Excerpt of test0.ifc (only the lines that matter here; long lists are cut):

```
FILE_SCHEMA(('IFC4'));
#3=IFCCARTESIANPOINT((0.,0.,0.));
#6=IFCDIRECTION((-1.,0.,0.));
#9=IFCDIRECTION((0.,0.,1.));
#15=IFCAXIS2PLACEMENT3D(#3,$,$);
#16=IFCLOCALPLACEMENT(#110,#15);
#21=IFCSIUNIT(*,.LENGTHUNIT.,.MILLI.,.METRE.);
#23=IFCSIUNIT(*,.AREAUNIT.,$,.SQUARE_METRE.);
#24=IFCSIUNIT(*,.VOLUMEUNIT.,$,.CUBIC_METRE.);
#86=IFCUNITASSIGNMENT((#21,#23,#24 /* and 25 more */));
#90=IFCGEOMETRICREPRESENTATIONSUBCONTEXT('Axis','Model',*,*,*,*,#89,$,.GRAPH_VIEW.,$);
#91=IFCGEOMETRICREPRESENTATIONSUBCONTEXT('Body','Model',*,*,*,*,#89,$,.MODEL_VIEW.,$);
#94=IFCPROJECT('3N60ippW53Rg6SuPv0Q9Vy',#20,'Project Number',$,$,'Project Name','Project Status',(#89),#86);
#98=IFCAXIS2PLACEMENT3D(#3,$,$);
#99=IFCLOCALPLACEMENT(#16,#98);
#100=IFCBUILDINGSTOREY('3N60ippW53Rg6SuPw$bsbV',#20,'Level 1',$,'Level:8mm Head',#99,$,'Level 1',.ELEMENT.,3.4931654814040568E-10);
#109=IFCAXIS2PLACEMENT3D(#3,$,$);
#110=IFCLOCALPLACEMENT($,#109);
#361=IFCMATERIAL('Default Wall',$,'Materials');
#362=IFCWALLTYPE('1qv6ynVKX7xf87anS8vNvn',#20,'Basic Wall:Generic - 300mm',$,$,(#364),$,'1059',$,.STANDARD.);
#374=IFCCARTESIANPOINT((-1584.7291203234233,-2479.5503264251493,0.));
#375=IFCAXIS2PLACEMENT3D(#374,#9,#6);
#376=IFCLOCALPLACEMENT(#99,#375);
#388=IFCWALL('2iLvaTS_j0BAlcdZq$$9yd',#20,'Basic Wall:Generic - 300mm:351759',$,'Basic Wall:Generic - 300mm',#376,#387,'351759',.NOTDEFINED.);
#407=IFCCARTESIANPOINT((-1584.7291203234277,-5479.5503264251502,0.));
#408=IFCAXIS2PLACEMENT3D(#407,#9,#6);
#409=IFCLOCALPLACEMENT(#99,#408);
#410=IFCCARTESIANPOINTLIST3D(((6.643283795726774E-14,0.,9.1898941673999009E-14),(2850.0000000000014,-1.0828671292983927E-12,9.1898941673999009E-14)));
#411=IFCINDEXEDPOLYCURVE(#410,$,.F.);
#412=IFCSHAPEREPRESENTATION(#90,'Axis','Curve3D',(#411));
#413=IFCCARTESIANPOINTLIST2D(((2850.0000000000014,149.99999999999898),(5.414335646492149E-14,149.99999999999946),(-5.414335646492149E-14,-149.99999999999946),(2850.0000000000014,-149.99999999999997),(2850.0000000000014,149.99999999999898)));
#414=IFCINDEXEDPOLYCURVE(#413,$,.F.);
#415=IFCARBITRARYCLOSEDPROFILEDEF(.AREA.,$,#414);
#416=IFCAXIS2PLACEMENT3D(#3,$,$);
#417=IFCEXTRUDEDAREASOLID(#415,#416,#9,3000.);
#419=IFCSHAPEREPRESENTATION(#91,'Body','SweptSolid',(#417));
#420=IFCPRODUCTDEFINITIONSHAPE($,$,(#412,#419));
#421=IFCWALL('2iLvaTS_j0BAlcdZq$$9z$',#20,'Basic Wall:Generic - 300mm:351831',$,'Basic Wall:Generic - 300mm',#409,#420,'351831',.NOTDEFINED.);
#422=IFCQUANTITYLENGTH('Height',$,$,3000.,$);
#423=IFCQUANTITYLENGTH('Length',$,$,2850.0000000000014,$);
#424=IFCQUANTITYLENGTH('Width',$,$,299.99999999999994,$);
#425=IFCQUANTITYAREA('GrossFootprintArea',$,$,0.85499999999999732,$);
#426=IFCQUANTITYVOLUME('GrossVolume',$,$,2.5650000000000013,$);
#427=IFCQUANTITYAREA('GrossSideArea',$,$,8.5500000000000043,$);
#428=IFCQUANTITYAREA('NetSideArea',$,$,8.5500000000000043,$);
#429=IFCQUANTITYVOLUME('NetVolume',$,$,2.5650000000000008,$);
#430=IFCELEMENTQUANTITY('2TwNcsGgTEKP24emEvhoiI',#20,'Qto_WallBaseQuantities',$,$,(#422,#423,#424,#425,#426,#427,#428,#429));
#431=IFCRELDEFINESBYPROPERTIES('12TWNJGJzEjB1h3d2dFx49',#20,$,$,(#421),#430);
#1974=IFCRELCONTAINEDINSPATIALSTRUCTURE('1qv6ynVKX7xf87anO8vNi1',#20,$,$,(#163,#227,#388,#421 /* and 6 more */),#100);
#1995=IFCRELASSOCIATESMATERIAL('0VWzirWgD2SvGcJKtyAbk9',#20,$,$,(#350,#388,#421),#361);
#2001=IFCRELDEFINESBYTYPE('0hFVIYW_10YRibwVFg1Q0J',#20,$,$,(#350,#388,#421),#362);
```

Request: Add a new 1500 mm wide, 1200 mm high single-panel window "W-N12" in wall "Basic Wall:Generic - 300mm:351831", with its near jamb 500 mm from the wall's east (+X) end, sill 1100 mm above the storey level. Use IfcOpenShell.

```python
import numpy as np
import ifcopenshell
import ifcopenshell.api.feature
import ifcopenshell.api.geometry
import ifcopenshell.api.pset
import ifcopenshell.api.root
import ifcopenshell.api.spatial
import ifcopenshell.geom
import ifcopenshell.util.element
import ifcopenshell.util.placement
import ifcopenshell.util.representation
import ifcopenshell.util.shape
import ifcopenshell.util.unit

model = ifcopenshell.open("test0.ifc")
unit_scale = ifcopenshell.util.unit.calculate_unit_scale(model)
area_scale = ifcopenshell.util.unit.calculate_unit_scale(model, "AREAUNIT")
volume_scale = ifcopenshell.util.unit.calculate_unit_scale(model, "VOLUMEUNIT")
settings = ifcopenshell.geom.settings()


def volume(element):
    """Net volume in cubic metres, openings subtracted."""
    shape = ifcopenshell.geom.create_shape(settings, element)
    return ifcopenshell.util.shape.get_volume(shape.geometry)


wall = model.by_guid("2iLvaTS_j0BAlcdZq$$9z$")
storey = ifcopenshell.util.element.get_container(wall, ifc_class="IfcBuildingStorey")
context = ifcopenshell.util.representation.get_context(model, "Model", "Body", "MODEL_VIEW")
before = volume(wall)

width, height, from_end, sill = 1.5, 1.2, 0.5, 1.1  # metres

# The wall runs along its own X axis, and the end named is its -X end.
wall_shape = ifcopenshell.geom.create_shape(settings, wall)
x, y, z = ifcopenshell.util.shape.get_vertices(wall_shape.geometry).T
start = x.min() + from_end
face, thickness = float(y.min()), float(y.max() - y.min())
wall_matrix = ifcopenshell.util.placement.get_local_placement(wall.ObjectPlacement)
level = ifcopenshell.util.placement.get_local_placement(storey.ObjectPlacement)[2, 3]


def in_wall(x, y):
    """Placement at x, y metres in the wall's axes, at sill height."""
    matrix = wall_matrix.copy()
    matrix[:, 3] = wall_matrix @ np.array([x / unit_scale, y / unit_scale, 0.0, 1.0])
    matrix[2, 3] = level + sill / unit_scale
    return matrix


# Opening: a box that overshoots both wall faces by 50 mm.
opening = ifcopenshell.api.root.create_entity(model, ifc_class="IfcOpeningElement", predefined_type="OPENING")
box = ifcopenshell.api.geometry.add_wall_representation(
    model, context=context, length=width, height=height, thickness=thickness + 0.1
)
ifcopenshell.api.geometry.assign_representation(model, product=opening, representation=box)
ifcopenshell.api.geometry.edit_object_placement(model, product=opening, matrix=in_wall(start, face - 0.05), is_si=False)
ifcopenshell.api.feature.add_feature(model, feature=opening, element=wall)

window = ifcopenshell.api.root.create_entity(model, ifc_class="IfcWindow", name="W-N12", predefined_type="WINDOW")
window.OverallWidth, window.OverallHeight = width / unit_scale, height / unit_scale
window.PartitioningType = "SINGLE_PANEL"
body = ifcopenshell.api.geometry.add_window_representation(
    model,
    context=context,
    overall_width=window.OverallWidth,
    overall_height=window.OverallHeight,
    partition_type="SINGLE_PANEL",
)
ifcopenshell.api.geometry.assign_representation(model, product=window, representation=body)
ifcopenshell.api.spatial.assign_container(model, products=[window], relating_structure=storey)
ifcopenshell.api.feature.add_filling(model, opening=opening, element=window)

# Centre the window in the wall's thickness.
ifcopenshell.api.geometry.edit_object_placement(model, product=window, matrix=in_wall(start, face), is_si=False)
window_shape = ifcopenshell.geom.create_shape(settings, window)
depth = ifcopenshell.util.shape.get_vertices(window_shape.geometry)[:, 1]
offset = face + thickness / 2 - (depth.min() + depth.max()) / 2
ifcopenshell.api.geometry.edit_object_placement(model, product=window, matrix=in_wall(start, offset), is_si=False)

after = volume(wall)

# Update the wall's stored quantities.
qto = model.by_id(ifcopenshell.util.element.get_pset(wall, "Qto_WallBaseQuantities", should_inherit=False)["id"])
ifcopenshell.api.pset.edit_qto(model, qto=qto, properties={
    "NetSideArea": after / thickness / area_scale,
    "NetVolume": after / volume_scale,
})

print(f"wall volume {before:.3f} -> {after:.3f} m3")

model.write("test0-out.ifc")
```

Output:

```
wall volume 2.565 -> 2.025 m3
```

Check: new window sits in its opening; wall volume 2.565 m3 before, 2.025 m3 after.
